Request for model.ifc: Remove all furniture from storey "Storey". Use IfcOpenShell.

First a look at what the model holds.

```python
import ifcopenshell
import ifcopenshell.util.element

model = ifcopenshell.open("model.ifc")
print(model.schema)
storey = next(s for s in model.by_type("IfcBuildingStorey") if s.Name == "Storey")
furniture = [e for e in ifcopenshell.util.element.get_decomposition(storey) if e.is_a("IfcFurnishingElement")]
seen = {}
for e in furniture:
    element_type = ifcopenshell.util.element.get_type(e)
    name = element_type.Name if element_type not in (None, e) else None
    seen[name] = seen.get(name, 0) + 1
for name, count in sorted(seen.items(), key=str):
    print(count, "x", name)
```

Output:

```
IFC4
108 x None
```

```python
import ifcopenshell
import ifcopenshell.api.root
import ifcopenshell.util.element

model = ifcopenshell.open("model.ifc")

storey = next(s for s in model.by_type("IfcBuildingStorey") if s.Name == "Storey")
furniture = [e for e in ifcopenshell.util.element.get_decomposition(storey) if e.is_a("IfcFurnishingElement")]

for e in furniture:
    ifcopenshell.api.root.remove_product(model, product=e)
print(len(furniture), "removed")

model.write("model_updated.ifc")
```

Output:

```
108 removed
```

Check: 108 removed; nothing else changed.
